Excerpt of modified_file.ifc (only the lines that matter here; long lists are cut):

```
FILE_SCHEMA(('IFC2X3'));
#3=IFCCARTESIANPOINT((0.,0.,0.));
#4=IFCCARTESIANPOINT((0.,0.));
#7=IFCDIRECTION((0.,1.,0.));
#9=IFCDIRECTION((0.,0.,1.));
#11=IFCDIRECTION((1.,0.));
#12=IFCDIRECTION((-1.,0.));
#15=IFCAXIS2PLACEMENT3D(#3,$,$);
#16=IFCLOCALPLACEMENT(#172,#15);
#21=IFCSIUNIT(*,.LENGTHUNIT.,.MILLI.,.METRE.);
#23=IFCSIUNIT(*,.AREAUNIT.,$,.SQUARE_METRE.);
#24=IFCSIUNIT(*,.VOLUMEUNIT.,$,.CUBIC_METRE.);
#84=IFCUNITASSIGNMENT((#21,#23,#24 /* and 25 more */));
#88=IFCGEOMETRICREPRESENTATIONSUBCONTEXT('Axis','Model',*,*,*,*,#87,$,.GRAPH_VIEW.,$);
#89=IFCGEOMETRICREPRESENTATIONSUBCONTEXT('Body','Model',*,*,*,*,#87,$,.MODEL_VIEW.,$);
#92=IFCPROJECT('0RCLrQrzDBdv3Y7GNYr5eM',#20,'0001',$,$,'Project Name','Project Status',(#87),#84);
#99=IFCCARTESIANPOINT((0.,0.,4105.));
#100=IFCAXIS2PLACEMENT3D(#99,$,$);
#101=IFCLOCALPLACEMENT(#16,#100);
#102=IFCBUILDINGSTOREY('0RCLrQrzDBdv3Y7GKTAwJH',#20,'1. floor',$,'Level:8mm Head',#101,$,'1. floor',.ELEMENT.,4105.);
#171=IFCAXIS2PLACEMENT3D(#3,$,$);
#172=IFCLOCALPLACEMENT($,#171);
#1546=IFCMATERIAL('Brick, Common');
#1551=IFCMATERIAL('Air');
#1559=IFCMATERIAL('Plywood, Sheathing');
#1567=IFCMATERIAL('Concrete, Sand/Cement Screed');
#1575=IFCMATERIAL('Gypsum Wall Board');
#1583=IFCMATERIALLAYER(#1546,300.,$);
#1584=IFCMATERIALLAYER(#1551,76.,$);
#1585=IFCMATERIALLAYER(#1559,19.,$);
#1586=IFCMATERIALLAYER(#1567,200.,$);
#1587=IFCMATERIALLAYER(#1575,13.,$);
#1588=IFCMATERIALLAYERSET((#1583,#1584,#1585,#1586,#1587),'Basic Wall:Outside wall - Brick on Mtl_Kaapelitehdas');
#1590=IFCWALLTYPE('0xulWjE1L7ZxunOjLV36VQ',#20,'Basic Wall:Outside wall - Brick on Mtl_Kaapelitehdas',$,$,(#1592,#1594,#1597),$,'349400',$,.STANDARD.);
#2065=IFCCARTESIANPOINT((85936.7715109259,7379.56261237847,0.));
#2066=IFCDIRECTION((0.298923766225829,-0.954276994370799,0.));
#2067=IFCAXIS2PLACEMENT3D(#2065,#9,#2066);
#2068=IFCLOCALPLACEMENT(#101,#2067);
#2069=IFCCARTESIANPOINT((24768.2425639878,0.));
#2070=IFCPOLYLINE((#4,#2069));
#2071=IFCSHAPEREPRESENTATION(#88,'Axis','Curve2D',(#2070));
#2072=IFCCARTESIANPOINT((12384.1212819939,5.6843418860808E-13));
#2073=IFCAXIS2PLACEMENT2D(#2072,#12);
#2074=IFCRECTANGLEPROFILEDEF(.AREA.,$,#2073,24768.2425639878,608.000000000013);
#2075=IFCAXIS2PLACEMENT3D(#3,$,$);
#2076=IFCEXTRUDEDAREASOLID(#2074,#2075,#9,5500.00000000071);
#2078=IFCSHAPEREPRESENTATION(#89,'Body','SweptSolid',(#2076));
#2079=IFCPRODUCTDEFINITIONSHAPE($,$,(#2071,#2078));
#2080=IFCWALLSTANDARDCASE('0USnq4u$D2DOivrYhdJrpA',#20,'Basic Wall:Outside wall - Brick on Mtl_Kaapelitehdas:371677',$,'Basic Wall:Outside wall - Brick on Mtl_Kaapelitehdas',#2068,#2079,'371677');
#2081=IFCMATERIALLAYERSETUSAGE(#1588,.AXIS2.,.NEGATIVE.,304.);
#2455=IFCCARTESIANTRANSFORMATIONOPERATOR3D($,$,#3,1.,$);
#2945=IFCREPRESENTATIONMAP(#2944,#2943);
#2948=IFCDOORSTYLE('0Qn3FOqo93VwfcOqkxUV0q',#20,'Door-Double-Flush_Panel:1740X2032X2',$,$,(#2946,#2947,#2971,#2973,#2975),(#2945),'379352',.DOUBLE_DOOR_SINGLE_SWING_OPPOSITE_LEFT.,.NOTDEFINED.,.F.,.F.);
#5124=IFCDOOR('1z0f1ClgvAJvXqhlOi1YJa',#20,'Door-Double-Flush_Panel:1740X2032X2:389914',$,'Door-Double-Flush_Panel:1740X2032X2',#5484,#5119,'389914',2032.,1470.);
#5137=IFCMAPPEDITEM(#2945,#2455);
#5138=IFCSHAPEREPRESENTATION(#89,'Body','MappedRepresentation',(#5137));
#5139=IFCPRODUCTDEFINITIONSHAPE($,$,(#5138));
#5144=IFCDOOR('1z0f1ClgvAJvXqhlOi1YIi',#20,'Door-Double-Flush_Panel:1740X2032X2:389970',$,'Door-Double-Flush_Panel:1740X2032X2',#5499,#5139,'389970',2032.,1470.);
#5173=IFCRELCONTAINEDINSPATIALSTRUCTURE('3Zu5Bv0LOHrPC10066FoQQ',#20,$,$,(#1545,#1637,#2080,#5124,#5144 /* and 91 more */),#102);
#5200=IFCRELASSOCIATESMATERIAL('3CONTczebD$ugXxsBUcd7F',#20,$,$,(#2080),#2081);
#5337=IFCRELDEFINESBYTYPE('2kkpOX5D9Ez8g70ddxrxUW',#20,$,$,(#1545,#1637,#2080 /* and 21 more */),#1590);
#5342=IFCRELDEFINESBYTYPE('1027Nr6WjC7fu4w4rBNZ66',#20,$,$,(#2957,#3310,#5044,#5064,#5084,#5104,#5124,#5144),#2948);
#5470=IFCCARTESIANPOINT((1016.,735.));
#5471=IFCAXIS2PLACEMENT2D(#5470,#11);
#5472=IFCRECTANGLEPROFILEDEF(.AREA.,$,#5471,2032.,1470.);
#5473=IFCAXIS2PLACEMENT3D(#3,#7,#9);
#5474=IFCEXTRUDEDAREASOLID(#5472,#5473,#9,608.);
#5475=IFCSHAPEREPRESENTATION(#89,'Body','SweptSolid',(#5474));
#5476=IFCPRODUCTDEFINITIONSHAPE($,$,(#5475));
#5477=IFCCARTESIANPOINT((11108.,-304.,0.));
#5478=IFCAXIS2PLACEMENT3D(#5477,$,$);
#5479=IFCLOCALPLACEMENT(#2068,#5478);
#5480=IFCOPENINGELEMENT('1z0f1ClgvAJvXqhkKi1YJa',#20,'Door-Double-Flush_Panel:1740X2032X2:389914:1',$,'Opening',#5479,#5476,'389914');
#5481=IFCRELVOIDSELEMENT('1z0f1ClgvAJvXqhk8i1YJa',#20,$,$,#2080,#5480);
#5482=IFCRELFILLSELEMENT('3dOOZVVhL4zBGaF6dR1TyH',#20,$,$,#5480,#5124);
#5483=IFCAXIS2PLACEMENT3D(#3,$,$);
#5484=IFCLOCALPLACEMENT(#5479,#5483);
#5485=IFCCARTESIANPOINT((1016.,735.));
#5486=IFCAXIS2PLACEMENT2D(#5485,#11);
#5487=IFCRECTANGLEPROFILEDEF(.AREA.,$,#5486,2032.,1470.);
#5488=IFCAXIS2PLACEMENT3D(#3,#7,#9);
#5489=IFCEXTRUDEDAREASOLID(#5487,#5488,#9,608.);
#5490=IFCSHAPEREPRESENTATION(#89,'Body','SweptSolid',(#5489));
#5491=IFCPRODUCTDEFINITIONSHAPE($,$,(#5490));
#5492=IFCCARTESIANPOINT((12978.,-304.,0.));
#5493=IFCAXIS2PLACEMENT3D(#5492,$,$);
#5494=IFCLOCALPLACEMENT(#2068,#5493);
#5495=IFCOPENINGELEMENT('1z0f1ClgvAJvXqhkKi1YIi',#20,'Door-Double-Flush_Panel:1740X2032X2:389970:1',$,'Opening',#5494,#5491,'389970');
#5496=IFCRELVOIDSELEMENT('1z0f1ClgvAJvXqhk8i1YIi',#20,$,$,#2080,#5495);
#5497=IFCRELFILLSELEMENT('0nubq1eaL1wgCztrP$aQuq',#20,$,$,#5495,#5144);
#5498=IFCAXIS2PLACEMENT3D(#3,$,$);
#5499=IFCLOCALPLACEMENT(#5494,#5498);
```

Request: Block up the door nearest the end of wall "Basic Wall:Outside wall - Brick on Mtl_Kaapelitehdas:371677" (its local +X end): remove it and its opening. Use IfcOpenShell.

```python
import ifcopenshell
import ifcopenshell.api.feature
import ifcopenshell.api.root
import ifcopenshell.geom
import ifcopenshell.util.shape

model = ifcopenshell.open("modified_file.ifc")
settings = ifcopenshell.geom.settings()


def volume(element):
    """Net volume in cubic metres, openings subtracted."""
    shape = ifcopenshell.geom.create_shape(settings, element)
    return ifcopenshell.util.shape.get_volume(shape.geometry)


door = model.by_guid("1z0f1ClgvAJvXqhlOi1YIi")
opening = door.FillsVoids[0].RelatingOpeningElement
wall = opening.VoidsElements[0].RelatingBuildingElement
before = volume(wall)

ifcopenshell.api.root.remove_product(model, product=door)
ifcopenshell.api.feature.remove_feature(model, feature=opening)

after = volume(wall)

print(f"wall volume {before:.3f} -> {after:.3f} m3")

model.write("modified_file-out.ifc")
```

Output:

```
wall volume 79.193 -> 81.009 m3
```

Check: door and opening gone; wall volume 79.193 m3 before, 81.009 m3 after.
